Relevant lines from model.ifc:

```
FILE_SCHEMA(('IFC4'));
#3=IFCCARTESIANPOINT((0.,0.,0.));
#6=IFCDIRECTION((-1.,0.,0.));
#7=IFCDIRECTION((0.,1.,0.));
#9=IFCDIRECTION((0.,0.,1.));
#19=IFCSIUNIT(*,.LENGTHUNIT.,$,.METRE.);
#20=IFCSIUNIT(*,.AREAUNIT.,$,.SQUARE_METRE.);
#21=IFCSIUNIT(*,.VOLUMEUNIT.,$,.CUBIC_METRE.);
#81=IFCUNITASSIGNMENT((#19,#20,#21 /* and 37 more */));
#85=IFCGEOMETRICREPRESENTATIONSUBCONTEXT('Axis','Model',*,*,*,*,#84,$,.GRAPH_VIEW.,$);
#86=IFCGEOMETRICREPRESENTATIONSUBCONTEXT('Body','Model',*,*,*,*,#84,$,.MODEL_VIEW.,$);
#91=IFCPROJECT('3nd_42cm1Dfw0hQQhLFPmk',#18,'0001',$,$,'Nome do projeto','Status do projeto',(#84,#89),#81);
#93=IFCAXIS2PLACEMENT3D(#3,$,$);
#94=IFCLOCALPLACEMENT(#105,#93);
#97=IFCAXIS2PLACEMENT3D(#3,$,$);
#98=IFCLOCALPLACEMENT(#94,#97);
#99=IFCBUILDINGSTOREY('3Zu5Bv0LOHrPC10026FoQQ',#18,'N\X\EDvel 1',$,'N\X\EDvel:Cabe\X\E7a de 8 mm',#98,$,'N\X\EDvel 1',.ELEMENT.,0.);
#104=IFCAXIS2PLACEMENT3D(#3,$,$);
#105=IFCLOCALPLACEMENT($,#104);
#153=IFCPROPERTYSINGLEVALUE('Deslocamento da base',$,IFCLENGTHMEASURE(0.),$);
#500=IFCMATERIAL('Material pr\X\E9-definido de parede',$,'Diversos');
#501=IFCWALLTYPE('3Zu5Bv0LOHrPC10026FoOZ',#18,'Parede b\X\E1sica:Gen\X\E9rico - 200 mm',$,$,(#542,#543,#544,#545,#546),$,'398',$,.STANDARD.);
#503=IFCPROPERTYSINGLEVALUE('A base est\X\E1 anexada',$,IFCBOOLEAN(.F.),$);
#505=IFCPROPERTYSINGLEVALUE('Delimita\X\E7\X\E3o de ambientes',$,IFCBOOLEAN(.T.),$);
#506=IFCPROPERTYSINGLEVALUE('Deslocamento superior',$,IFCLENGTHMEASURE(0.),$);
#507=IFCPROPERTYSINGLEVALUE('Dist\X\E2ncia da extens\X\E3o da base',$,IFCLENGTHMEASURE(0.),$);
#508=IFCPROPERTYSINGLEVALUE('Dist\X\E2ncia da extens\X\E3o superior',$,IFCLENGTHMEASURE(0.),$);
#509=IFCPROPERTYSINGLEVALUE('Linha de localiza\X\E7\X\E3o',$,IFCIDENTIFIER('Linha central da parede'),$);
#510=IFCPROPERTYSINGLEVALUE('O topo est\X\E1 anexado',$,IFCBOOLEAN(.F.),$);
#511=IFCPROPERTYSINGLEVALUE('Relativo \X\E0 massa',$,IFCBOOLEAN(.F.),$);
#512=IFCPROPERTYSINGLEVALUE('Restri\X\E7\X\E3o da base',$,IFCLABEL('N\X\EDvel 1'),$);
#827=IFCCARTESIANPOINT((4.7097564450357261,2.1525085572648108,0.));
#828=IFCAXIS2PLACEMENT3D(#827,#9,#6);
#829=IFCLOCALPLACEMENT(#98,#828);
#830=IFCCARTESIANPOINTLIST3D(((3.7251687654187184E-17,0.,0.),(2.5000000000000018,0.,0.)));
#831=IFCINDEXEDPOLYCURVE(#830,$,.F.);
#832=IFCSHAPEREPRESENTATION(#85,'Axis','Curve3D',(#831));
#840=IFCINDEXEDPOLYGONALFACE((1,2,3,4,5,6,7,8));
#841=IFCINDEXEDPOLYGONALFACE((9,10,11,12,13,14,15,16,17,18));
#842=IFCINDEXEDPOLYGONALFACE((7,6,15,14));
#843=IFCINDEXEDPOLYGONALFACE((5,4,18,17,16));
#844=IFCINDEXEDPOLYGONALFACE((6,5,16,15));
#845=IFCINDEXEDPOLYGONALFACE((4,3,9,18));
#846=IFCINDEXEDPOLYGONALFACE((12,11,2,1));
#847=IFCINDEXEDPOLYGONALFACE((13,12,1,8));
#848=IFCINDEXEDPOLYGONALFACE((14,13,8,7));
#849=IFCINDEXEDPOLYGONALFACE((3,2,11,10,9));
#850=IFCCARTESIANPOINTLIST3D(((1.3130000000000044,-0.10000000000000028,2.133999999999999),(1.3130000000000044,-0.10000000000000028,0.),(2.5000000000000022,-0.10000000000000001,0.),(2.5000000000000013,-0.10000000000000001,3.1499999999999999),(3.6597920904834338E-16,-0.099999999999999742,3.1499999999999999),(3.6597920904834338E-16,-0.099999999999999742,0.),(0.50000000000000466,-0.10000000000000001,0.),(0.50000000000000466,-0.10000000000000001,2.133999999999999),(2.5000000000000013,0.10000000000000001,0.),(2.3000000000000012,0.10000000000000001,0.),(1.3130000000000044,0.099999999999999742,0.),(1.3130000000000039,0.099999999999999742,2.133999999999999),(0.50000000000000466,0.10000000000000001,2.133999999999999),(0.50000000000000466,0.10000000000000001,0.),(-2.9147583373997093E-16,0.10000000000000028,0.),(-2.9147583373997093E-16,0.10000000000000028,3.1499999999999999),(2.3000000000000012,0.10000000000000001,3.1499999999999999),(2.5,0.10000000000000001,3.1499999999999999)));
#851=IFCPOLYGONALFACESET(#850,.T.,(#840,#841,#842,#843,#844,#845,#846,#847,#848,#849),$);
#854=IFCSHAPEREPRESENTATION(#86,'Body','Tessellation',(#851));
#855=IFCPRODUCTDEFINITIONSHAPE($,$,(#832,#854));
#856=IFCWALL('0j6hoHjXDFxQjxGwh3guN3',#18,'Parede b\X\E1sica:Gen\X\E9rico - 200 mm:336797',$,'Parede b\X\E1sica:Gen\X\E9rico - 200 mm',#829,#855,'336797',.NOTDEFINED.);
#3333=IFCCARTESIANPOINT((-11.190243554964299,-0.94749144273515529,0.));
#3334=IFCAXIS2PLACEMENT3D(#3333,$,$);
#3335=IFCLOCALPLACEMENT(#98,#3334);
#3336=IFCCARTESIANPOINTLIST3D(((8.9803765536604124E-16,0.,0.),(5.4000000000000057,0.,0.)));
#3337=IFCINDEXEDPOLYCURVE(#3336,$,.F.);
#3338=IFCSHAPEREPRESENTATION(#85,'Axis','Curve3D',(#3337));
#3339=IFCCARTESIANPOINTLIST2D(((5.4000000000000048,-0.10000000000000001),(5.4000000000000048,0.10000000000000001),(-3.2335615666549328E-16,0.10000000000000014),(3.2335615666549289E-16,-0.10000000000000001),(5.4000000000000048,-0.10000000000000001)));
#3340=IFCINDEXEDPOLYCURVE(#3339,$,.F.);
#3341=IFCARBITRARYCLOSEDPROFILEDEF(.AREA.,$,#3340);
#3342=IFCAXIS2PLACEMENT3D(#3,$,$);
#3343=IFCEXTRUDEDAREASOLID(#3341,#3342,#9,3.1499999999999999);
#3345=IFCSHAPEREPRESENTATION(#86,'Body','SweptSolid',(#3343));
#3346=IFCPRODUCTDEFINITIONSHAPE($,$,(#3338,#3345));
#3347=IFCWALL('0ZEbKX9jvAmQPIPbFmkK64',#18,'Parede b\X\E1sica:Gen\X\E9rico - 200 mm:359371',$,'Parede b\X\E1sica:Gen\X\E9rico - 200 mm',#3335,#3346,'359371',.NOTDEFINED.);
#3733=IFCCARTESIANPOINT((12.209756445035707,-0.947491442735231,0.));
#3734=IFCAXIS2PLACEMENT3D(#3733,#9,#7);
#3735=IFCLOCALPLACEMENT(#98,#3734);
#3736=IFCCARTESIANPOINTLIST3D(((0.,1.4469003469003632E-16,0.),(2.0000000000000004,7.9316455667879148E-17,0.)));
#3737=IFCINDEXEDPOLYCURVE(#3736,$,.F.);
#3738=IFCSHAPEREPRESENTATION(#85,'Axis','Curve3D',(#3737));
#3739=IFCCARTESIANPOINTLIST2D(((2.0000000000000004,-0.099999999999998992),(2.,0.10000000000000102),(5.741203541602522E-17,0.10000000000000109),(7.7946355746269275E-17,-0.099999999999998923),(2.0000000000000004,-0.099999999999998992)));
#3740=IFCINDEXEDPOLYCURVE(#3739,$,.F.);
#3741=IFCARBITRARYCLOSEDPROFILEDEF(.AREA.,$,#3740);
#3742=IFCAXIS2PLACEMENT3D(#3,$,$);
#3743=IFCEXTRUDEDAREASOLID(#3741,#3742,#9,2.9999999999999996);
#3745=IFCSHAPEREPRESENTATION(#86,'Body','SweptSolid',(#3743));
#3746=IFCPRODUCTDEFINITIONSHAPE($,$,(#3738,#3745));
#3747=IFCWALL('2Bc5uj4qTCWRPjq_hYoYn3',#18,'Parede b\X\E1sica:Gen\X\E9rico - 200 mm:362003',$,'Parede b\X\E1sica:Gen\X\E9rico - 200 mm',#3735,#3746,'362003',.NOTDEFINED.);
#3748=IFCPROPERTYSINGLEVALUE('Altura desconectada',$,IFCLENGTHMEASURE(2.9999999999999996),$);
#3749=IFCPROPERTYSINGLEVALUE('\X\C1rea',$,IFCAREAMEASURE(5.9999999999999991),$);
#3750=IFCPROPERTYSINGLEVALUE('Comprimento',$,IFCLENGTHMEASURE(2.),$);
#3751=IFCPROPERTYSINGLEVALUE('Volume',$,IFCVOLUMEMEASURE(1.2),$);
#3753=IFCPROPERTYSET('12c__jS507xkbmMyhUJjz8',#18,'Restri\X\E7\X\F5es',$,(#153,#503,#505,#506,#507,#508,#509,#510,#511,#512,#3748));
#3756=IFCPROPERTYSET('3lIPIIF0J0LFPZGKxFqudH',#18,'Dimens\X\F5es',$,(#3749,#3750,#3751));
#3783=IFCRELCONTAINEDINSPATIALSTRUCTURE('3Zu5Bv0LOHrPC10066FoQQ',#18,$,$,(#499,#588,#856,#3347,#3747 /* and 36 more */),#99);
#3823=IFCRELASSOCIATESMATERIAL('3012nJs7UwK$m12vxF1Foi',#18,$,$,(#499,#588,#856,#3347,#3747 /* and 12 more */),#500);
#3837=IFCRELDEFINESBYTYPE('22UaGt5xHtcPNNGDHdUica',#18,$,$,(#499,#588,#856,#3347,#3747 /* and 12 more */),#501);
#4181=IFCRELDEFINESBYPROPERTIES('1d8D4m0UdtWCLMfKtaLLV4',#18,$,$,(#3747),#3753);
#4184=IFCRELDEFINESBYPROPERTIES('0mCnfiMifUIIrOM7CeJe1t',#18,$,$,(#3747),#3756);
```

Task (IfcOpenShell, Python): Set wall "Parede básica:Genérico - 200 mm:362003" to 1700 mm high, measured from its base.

```python
import ifcopenshell
import ifcopenshell.api.pset
import ifcopenshell.geom
import ifcopenshell.util.element
import ifcopenshell.util.representation
import ifcopenshell.util.shape
import ifcopenshell.util.unit

model = ifcopenshell.open("model.ifc")
area_scale = ifcopenshell.util.unit.calculate_unit_scale(model, "AREAUNIT")
volume_scale = ifcopenshell.util.unit.calculate_unit_scale(model, "VOLUMEUNIT")
settings = ifcopenshell.geom.settings()


def volume(element):
    """Net volume in cubic metres, openings subtracted."""
    shape = ifcopenshell.geom.create_shape(settings, element)
    return ifcopenshell.util.shape.get_volume(shape.geometry)


wall = model.by_guid("2Bc5uj4qTCWRPjq_hYoYn3")
before = volume(wall)

body = ifcopenshell.util.representation.get_representation(wall, "Model", "Body")
solid = body.Items[0]
old_height = solid.Depth
solid.Depth = 1.7
after = volume(wall)
thickness = 0.2  # wall thickness in metres

# Update the stored height, areas and volumes.
pset = model.by_id(ifcopenshell.util.element.get_pset(wall, "Restrições", should_inherit=False)["id"])
ifcopenshell.api.pset.edit_pset(model, pset=pset, properties={
    "Altura desconectada": model.create_entity("IfcLengthMeasure", solid.Depth),
})
pset = model.by_id(ifcopenshell.util.element.get_pset(wall, "Dimensões", should_inherit=False)["id"])
ifcopenshell.api.pset.edit_pset(model, pset=pset, properties={
    "Área": model.create_entity("IfcAreaMeasure", after / thickness / area_scale),
    "Volume": model.create_entity("IfcVolumeMeasure", after / volume_scale),
})

print(f"height {old_height:g} -> {solid.Depth:g}, volume {before:.3f} -> {after:.3f} m3")

model.write("model-out.ifc")
```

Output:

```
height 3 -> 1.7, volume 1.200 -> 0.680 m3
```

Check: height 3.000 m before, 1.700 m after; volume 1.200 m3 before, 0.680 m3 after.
